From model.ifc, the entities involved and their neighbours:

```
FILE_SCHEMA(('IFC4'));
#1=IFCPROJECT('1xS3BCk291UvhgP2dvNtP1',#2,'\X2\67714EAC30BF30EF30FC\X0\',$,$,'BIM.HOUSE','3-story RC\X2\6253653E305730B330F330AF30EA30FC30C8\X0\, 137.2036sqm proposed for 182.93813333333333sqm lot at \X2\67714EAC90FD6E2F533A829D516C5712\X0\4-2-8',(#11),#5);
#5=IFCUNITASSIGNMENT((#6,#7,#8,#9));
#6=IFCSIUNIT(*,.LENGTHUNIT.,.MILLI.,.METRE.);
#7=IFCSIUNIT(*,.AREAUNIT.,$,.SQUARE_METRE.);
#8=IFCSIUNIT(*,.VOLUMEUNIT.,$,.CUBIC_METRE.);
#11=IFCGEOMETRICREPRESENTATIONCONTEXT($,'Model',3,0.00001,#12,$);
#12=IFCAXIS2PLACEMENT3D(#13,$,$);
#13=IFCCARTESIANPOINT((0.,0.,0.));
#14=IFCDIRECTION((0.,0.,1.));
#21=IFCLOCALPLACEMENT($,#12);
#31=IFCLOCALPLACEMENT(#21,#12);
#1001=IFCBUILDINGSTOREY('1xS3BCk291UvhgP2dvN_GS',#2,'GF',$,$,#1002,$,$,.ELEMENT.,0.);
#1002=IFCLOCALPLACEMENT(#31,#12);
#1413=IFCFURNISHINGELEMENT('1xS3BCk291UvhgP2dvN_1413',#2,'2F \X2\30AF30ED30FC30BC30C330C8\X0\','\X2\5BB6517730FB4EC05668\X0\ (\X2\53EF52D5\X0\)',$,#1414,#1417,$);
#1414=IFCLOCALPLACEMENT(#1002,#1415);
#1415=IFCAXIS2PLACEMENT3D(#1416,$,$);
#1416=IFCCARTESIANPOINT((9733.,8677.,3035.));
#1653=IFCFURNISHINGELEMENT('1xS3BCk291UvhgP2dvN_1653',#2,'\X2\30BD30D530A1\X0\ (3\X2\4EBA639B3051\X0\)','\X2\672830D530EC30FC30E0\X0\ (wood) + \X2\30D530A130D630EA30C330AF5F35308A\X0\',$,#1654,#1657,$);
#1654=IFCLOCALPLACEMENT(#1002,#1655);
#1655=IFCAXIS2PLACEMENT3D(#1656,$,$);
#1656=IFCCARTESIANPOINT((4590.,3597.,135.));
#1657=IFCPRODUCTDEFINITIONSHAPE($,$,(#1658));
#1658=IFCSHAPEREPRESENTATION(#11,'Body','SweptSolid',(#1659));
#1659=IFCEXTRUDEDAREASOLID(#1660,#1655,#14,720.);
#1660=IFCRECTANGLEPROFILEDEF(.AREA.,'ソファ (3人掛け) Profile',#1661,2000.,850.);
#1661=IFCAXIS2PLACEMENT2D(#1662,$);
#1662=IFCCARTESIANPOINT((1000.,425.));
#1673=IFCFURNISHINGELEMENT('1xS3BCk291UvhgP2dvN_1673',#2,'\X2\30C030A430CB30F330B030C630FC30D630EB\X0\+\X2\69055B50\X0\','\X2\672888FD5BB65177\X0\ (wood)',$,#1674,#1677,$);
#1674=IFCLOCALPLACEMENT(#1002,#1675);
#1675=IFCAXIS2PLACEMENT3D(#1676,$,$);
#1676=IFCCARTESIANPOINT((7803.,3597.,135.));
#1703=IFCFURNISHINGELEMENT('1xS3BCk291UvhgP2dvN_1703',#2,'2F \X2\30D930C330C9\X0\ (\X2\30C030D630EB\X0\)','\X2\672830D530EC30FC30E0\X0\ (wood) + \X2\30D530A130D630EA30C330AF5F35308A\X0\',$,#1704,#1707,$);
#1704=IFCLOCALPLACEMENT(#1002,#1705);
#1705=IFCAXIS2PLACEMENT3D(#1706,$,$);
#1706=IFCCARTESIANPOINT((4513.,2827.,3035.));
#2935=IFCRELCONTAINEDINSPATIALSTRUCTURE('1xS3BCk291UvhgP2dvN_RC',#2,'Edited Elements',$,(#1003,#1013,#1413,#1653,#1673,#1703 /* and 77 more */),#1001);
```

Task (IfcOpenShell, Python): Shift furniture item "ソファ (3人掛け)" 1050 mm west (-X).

```python
import ifcopenshell
import ifcopenshell.api.geometry
import ifcopenshell.util.placement
import ifcopenshell.util.unit

model = ifcopenshell.open("model.ifc")
unit_scale = ifcopenshell.util.unit.calculate_unit_scale(model)

item = model.by_guid("1xS3BCk291UvhgP2dvN_1653")
matrix = ifcopenshell.util.placement.get_local_placement(item.ObjectPlacement)
matrix[0, 3] -= 1.05 / unit_scale
ifcopenshell.api.geometry.edit_object_placement(model, product=item, matrix=matrix, is_si=False)

print(ifcopenshell.util.placement.get_local_placement(item.ObjectPlacement).round(3) + 0.0)

model.write("model_rev.ifc")
```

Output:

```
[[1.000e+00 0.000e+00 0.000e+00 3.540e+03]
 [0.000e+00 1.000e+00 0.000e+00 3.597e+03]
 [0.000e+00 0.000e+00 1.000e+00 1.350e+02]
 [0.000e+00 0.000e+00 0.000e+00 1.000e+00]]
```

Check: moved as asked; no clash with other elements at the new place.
